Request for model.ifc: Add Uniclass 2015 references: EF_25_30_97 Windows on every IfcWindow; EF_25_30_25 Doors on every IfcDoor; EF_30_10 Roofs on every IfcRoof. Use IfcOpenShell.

First a look at what the model holds.

```python
import ifcopenshell

model = ifcopenshell.open("model.ifc")
print(model.schema)
print("classifications:", [c.Name for c in model.by_type("IfcClassification")])
for ifc_class in ("IfcDoor", "IfcRoof", "IfcStair", "IfcWall", "IfcWindow"):
    print(ifc_class, len(model.by_type(ifc_class)))
```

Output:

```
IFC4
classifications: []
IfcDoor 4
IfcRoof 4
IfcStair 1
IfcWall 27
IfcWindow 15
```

```python
import ifcopenshell
import ifcopenshell.api.classification

model = ifcopenshell.open("model.ifc")

system = ifcopenshell.api.classification.add_classification(model, classification="Uniclass 2015")

codes = {
    "IfcWindow": ("EF_25_30_97", "Windows"),
    "IfcDoor": ("EF_25_30_25", "Doors"),
    "IfcRoof": ("EF_30_10", "Roofs"),
}
for ifc_class, (code, name) in codes.items():
    products = model.by_type(ifc_class)
    ifcopenshell.api.classification.add_reference(
        model, products=products, classification=system, identification=code, name=name
    )
    print(code, len(products))

model.write("model_edited.ifc")
```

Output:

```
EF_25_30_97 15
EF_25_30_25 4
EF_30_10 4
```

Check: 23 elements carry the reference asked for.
